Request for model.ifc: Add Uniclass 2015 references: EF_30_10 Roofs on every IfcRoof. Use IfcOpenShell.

First a look at what the model holds.

```python
import ifcopenshell

model = ifcopenshell.open("model.ifc")
print(model.schema)
print("classifications:", [c.Name for c in model.by_type("IfcClassification")])
for ifc_class in ("IfcDoor", "IfcRoof", "IfcStair", "IfcWall", "IfcWindow"):
    print(ifc_class, len(model.by_type(ifc_class)))
```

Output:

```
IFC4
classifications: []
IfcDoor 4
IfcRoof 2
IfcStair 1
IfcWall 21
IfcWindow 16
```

```python
import ifcopenshell
import ifcopenshell.api.classification

model = ifcopenshell.open("model.ifc")

system = ifcopenshell.api.classification.add_classification(model, classification="Uniclass 2015")

codes = {
    "IfcRoof": ("EF_30_10", "Roofs"),
}
for ifc_class, (code, name) in codes.items():
    products = model.by_type(ifc_class)
    ifcopenshell.api.classification.add_reference(
        model, products=products, classification=system, identification=code, name=name
    )
    print(code, len(products))

model.write("model_edited.ifc")
```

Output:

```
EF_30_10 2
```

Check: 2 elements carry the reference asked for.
